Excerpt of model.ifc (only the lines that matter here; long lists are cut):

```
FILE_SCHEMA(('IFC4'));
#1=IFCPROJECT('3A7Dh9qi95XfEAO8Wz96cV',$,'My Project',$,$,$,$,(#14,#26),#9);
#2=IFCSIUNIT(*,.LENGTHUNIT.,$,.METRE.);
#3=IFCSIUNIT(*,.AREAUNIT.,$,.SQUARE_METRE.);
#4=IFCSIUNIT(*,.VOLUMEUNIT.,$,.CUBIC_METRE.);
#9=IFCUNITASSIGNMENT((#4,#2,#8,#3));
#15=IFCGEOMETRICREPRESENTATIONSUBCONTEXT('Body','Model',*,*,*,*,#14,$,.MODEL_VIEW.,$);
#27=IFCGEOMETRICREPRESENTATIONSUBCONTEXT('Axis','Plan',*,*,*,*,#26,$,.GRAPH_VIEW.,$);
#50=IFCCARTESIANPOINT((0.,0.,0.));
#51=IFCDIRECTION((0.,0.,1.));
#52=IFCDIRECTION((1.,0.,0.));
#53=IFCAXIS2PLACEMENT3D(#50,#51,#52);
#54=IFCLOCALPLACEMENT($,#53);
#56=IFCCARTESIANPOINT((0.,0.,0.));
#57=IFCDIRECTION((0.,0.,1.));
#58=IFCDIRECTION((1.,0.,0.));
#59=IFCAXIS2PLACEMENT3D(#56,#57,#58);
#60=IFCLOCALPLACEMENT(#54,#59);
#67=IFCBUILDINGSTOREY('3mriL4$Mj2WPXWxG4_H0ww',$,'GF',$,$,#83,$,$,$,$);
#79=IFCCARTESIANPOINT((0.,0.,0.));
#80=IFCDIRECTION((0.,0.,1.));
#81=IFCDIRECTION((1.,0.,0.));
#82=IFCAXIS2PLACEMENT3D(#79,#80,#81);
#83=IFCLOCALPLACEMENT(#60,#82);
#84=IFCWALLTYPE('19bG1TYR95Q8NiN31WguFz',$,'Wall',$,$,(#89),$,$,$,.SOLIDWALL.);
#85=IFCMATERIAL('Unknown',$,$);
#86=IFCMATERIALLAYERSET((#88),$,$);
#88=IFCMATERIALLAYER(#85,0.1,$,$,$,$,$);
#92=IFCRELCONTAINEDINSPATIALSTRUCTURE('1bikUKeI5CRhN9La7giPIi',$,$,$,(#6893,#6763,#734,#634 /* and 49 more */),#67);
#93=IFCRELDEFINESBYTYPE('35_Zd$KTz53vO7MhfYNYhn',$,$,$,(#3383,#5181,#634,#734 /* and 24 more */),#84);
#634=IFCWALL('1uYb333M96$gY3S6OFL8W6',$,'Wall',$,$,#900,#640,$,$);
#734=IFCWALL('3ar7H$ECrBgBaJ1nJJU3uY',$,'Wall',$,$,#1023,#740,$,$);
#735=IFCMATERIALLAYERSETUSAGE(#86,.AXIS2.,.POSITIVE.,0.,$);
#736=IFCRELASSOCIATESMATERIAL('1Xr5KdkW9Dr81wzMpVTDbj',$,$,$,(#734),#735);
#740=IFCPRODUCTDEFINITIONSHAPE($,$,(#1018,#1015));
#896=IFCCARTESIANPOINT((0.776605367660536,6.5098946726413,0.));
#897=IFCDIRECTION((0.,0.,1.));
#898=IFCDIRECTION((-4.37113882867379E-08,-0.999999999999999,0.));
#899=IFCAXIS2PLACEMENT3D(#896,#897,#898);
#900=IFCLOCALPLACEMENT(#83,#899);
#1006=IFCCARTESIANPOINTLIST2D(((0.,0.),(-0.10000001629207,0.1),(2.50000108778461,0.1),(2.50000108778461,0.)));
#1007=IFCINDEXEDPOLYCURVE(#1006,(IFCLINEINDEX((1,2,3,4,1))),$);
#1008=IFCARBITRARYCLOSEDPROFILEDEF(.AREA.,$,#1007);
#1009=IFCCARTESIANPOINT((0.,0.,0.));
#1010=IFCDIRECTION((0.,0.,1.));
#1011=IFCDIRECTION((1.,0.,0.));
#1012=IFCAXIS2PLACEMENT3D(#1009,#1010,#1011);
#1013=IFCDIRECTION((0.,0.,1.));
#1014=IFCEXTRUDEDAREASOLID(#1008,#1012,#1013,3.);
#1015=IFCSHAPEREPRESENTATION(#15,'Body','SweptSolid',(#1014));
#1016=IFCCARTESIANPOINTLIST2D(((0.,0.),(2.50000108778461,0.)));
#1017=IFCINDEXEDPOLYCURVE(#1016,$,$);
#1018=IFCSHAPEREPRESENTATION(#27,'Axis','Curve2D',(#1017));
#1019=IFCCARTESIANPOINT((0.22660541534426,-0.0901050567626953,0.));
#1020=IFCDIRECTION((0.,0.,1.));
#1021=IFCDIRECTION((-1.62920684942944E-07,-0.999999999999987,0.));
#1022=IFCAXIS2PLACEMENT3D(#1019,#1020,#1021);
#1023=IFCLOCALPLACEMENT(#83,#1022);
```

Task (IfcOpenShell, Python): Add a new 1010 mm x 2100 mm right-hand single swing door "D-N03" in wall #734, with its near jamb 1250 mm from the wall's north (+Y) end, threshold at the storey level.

```python
import numpy as np
import ifcopenshell
import ifcopenshell.api.feature
import ifcopenshell.api.geometry
import ifcopenshell.api.root
import ifcopenshell.api.spatial
import ifcopenshell.geom
import ifcopenshell.util.element
import ifcopenshell.util.placement
import ifcopenshell.util.representation
import ifcopenshell.util.shape
import ifcopenshell.util.unit

model = ifcopenshell.open("model.ifc")
unit_scale = ifcopenshell.util.unit.calculate_unit_scale(model)
settings = ifcopenshell.geom.settings()


def volume(element):
    """Net volume in cubic metres, openings subtracted."""
    shape = ifcopenshell.geom.create_shape(settings, element)
    return ifcopenshell.util.shape.get_volume(shape.geometry)


wall = model.by_guid("3ar7H$ECrBgBaJ1nJJU3uY")
storey = ifcopenshell.util.element.get_container(wall, ifc_class="IfcBuildingStorey")
context = ifcopenshell.util.representation.get_context(model, "Model", "Body", "MODEL_VIEW")
before = volume(wall)

width, height, from_end, sill = 1.01, 2.1, 1.25, 0.0  # metres

# The wall runs along its own X axis, and the end named is its -X end.
wall_shape = ifcopenshell.geom.create_shape(settings, wall)
x, y, z = ifcopenshell.util.shape.get_vertices(wall_shape.geometry).T
start = x.min() + from_end
face, thickness = float(y.min()), float(y.max() - y.min())
wall_matrix = ifcopenshell.util.placement.get_local_placement(wall.ObjectPlacement)
level = ifcopenshell.util.placement.get_local_placement(storey.ObjectPlacement)[2, 3]


def in_wall(x, y):
    """Placement at x, y metres in the wall's axes, at sill height."""
    matrix = wall_matrix.copy()
    matrix[:, 3] = wall_matrix @ np.array([x / unit_scale, y / unit_scale, 0.0, 1.0])
    matrix[2, 3] = level + sill / unit_scale
    return matrix


# Opening: a box that overshoots both wall faces by 50 mm.
opening = ifcopenshell.api.root.create_entity(model, ifc_class="IfcOpeningElement", predefined_type="OPENING")
box = ifcopenshell.api.geometry.add_wall_representation(
    model, context=context, length=width, height=height, thickness=thickness + 0.1
)
ifcopenshell.api.geometry.assign_representation(model, product=opening, representation=box)
ifcopenshell.api.geometry.edit_object_placement(model, product=opening, matrix=in_wall(start, face - 0.05), is_si=False)
ifcopenshell.api.feature.add_feature(model, feature=opening, element=wall)

door = ifcopenshell.api.root.create_entity(model, ifc_class="IfcDoor", name="D-N03", predefined_type="DOOR")
door.OverallWidth, door.OverallHeight = width / unit_scale, height / unit_scale
door.OperationType = "SINGLE_SWING_RIGHT"
body = ifcopenshell.api.geometry.add_door_representation(
    model,
    context=context,
    overall_width=door.OverallWidth,
    overall_height=door.OverallHeight,
    operation_type="SINGLE_SWING_RIGHT",
    lining_properties={"LiningDepth": thickness / unit_scale, "ThresholdDepth": thickness / unit_scale},
)
ifcopenshell.api.geometry.assign_representation(model, product=door, representation=body)
ifcopenshell.api.spatial.assign_container(model, products=[door], relating_structure=storey)
ifcopenshell.api.feature.add_filling(model, opening=opening, element=door)

# The lining spans the wall, so the door starts at the wall face.
ifcopenshell.api.geometry.edit_object_placement(model, product=door, matrix=in_wall(start, face), is_si=False)

after = volume(wall)

print(f"wall volume {before:.3f} -> {after:.3f} m3")

model.write("model_edited.ifc")
```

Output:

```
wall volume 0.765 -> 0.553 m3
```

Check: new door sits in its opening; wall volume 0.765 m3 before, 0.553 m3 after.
